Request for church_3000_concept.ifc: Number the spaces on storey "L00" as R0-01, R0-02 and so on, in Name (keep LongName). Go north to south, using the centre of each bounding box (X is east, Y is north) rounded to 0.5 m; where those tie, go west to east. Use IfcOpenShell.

First a look at what the model holds.

```python
import ifcopenshell
import ifcopenshell.util.element
import ifcopenshell.util.placement

model = ifcopenshell.open("church_3000_concept.ifc")
print(model.schema)
storey = next(s for s in model.by_type("IfcBuildingStorey") if s.Name == "L00")
spaces = [e for e in ifcopenshell.util.element.get_decomposition(storey) if e.is_a("IfcSpace")]
for e in sorted(spaces, key=lambda e: e.id()):
    origin = ifcopenshell.util.placement.get_local_placement(e.ObjectPlacement)[:3, 3]
    print(e.id(), e.Name, e.LongName, origin.round(2) + 0.0, sep=" | ")
```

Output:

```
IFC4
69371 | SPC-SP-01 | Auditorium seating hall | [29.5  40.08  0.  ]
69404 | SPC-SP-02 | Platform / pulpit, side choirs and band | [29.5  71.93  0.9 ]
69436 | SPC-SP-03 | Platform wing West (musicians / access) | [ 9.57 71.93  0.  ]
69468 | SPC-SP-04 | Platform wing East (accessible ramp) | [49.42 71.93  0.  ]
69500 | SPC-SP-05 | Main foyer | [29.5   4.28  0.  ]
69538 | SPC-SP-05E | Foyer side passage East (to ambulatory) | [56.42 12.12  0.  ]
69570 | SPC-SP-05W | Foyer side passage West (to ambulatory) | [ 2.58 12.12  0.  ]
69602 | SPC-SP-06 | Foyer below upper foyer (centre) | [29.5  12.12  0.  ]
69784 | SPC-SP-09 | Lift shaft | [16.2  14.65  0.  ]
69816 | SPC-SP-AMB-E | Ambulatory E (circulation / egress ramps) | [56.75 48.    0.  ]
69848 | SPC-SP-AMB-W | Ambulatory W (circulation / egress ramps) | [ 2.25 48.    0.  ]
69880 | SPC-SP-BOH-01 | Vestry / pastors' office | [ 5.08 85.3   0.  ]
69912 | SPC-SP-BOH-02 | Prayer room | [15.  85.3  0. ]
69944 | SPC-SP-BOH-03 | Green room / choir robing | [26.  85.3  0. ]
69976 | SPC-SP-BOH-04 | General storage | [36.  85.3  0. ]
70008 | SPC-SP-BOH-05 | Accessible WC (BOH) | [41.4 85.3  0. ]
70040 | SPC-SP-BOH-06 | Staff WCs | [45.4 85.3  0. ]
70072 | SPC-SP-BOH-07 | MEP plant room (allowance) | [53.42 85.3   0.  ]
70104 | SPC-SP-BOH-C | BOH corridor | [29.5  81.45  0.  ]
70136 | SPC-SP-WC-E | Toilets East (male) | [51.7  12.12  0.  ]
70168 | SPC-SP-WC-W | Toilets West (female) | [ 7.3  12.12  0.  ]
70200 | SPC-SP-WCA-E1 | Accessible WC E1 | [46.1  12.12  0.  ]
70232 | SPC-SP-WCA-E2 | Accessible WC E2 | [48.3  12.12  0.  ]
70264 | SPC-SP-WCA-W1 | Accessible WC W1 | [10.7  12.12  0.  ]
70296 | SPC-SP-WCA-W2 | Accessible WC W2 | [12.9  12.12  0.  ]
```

```python
import ifcopenshell
import ifcopenshell.geom
import ifcopenshell.util.element
import ifcopenshell.util.shape

model = ifcopenshell.open("church_3000_concept.ifc")
settings = ifcopenshell.geom.settings()
settings.set("use-world-coords", True)


def centre(element):
    shape = ifcopenshell.geom.create_shape(settings, element)
    return ifcopenshell.util.shape.get_bbox_centroid(shape.geometry)


storey = next(s for s in model.by_type("IfcBuildingStorey") if s.Name == "L00")
spaces = [e for e in ifcopenshell.util.element.get_decomposition(storey) if e.is_a("IfcSpace")]

# Insertion points can sit at a corner or the storey origin, so sort by the geometry (in metres).
centres = {e: centre(e) for e in spaces}
spaces.sort(key=lambda e: (-round(centres[e][1] / 0.5), centres[e][0]))

for i, e in enumerate(spaces, start=1):
    number = f"R0-{i:02d}"
    e.Name = number
    print(e.id(), number)

model.write("church_3000_concept_edited.ifc")
```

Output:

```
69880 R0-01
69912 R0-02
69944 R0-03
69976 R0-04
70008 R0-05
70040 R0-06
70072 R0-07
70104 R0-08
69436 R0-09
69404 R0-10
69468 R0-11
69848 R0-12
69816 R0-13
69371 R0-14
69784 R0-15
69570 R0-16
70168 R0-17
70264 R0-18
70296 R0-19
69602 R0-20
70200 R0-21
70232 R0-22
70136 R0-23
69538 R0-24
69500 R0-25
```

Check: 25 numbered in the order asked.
